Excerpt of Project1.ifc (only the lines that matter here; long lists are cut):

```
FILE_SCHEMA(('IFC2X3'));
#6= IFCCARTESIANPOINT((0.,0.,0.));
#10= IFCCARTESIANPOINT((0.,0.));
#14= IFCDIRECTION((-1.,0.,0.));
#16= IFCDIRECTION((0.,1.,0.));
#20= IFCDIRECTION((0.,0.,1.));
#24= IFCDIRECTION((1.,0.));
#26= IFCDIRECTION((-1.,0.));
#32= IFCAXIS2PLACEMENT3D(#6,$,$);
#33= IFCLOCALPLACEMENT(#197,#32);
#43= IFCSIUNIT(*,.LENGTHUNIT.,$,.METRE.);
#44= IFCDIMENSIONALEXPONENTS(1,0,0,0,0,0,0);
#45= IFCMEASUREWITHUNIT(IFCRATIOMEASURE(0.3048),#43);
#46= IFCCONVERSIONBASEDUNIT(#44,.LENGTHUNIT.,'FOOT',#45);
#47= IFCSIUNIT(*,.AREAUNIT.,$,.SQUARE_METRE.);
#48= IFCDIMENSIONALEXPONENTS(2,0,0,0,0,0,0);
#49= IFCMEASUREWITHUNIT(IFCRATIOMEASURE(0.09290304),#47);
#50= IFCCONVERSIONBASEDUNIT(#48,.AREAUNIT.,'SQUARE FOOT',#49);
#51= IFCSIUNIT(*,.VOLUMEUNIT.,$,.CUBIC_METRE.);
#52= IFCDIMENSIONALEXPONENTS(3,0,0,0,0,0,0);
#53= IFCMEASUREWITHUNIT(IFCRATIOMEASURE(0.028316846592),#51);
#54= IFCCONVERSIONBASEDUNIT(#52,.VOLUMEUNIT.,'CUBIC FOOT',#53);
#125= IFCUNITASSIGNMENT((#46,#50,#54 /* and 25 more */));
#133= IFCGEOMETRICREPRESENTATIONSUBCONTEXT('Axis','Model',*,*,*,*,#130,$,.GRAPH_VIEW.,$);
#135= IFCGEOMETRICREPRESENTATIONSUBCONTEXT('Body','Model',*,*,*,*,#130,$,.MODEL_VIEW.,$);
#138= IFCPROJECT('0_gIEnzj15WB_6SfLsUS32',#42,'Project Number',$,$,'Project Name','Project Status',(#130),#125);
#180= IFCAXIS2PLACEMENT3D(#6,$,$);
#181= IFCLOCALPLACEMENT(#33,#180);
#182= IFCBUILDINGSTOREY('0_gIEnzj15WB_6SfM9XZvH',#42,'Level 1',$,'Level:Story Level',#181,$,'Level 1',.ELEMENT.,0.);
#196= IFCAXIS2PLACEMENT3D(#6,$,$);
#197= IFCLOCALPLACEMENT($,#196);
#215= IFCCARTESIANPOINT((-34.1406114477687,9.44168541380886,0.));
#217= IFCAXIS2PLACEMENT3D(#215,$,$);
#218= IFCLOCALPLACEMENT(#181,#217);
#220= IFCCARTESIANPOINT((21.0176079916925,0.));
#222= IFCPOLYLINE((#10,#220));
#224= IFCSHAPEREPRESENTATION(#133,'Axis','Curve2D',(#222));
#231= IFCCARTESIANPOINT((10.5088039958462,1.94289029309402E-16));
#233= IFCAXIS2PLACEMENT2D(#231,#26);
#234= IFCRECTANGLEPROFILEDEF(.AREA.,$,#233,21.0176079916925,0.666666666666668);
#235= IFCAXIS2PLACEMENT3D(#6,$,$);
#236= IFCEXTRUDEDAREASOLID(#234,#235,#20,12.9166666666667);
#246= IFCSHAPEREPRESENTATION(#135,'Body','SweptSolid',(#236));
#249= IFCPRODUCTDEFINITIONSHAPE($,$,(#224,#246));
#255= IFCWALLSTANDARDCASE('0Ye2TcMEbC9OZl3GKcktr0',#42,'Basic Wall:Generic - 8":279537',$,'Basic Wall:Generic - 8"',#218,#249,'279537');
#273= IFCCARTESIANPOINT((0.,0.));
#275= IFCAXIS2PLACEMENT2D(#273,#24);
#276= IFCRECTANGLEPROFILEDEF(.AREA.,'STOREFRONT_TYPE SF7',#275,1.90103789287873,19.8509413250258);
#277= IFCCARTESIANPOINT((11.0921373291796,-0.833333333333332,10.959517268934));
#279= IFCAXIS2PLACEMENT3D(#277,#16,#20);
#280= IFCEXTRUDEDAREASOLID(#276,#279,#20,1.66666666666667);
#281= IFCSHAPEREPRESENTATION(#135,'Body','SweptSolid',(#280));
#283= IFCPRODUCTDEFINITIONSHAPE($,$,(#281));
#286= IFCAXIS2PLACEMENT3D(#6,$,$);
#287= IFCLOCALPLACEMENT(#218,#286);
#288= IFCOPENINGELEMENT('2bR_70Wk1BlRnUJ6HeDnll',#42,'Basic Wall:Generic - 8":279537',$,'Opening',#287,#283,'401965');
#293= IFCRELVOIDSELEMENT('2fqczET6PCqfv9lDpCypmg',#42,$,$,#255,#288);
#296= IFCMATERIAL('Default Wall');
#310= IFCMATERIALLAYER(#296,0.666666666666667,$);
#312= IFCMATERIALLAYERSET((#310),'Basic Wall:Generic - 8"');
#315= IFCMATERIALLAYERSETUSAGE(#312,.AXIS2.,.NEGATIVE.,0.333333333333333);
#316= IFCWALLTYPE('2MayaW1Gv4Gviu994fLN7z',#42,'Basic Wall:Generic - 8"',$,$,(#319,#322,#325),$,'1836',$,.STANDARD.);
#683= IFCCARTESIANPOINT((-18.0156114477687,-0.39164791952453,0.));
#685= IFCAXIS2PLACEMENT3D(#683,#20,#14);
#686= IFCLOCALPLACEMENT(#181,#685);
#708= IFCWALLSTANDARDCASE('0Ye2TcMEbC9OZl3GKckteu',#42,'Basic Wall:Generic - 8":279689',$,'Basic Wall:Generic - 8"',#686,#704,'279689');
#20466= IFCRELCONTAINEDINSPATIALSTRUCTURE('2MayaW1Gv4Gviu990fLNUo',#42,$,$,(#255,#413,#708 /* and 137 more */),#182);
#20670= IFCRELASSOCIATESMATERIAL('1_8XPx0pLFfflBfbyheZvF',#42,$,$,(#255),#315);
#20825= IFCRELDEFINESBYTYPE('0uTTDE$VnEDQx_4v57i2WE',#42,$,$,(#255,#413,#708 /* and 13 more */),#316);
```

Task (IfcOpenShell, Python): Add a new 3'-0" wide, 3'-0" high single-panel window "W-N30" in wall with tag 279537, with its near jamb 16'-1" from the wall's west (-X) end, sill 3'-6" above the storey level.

```python
import numpy as np
import ifcopenshell
import ifcopenshell.api.feature
import ifcopenshell.api.geometry
import ifcopenshell.api.root
import ifcopenshell.api.spatial
import ifcopenshell.api.type
import ifcopenshell.geom
import ifcopenshell.util.element
import ifcopenshell.util.placement
import ifcopenshell.util.representation
import ifcopenshell.util.shape
import ifcopenshell.util.unit

model = ifcopenshell.open("Project1.ifc")
unit_scale = ifcopenshell.util.unit.calculate_unit_scale(model)
settings = ifcopenshell.geom.settings()


def volume(element):
    """Net volume in cubic metres, openings subtracted."""
    shape = ifcopenshell.geom.create_shape(settings, element)
    return ifcopenshell.util.shape.get_volume(shape.geometry)


wall = model.by_guid("0Ye2TcMEbC9OZl3GKcktr0")
storey = ifcopenshell.util.element.get_container(wall, ifc_class="IfcBuildingStorey")
context = ifcopenshell.util.representation.get_context(model, "Model", "Body", "MODEL_VIEW")
before = volume(wall)

width, height, from_end, sill = 0.9144, 0.9144, 4.9022, 1.0668  # metres

# The wall runs along its own X axis, and the end named is its -X end.
wall_shape = ifcopenshell.geom.create_shape(settings, wall)
x, y, z = ifcopenshell.util.shape.get_vertices(wall_shape.geometry).T
start = x.min() + from_end
face, thickness = float(y.min()), float(y.max() - y.min())
wall_matrix = ifcopenshell.util.placement.get_local_placement(wall.ObjectPlacement)
level = ifcopenshell.util.placement.get_local_placement(storey.ObjectPlacement)[2, 3]


def in_wall(x, y):
    """Placement at x, y metres in the wall's axes, at sill height."""
    matrix = wall_matrix.copy()
    matrix[:, 3] = wall_matrix @ np.array([x / unit_scale, y / unit_scale, 0.0, 1.0])
    matrix[2, 3] = level + sill / unit_scale
    return matrix


# Opening: a box that overshoots both wall faces by 50 mm.
opening = ifcopenshell.api.root.create_entity(model, ifc_class="IfcOpeningElement")
box = ifcopenshell.api.geometry.add_wall_representation(
    model, context=context, length=width, height=height, thickness=thickness + 0.1
)
ifcopenshell.api.geometry.assign_representation(model, product=opening, representation=box)
ifcopenshell.api.geometry.edit_object_placement(model, product=opening, matrix=in_wall(start, face - 0.05), is_si=False)
ifcopenshell.api.feature.add_feature(model, feature=opening, element=wall)

window = ifcopenshell.api.root.create_entity(model, ifc_class="IfcWindow", name="W-N30")
window.OverallWidth, window.OverallHeight = width / unit_scale, height / unit_scale
body = ifcopenshell.api.geometry.add_window_representation(
    model,
    context=context,
    overall_width=window.OverallWidth,
    overall_height=window.OverallHeight,
    partition_type="SINGLE_PANEL",
)
ifcopenshell.api.geometry.assign_representation(model, product=window, representation=body)
ifcopenshell.api.spatial.assign_container(model, products=[window], relating_structure=storey)
fills = ifcopenshell.api.feature.add_filling(model, opening=opening, element=window)
fills.OwnerHistory = window.OwnerHistory  # required in IFC2X3

# IFC2X3 keeps the operation on the window style.
style = ifcopenshell.api.root.create_entity(model, ifc_class="IfcWindowStyle", name="W-N30")
style.OperationType, style.ConstructionType = "SINGLE_PANEL", "NOTDEFINED"
style.ParameterTakesPrecedence = style.Sizeable = False
ifcopenshell.api.type.assign_type(model, related_objects=[window], relating_type=style)

# Centre the window in the wall's thickness.
ifcopenshell.api.geometry.edit_object_placement(model, product=window, matrix=in_wall(start, face), is_si=False)
window_shape = ifcopenshell.geom.create_shape(settings, window)
depth = ifcopenshell.util.shape.get_vertices(window_shape.geometry)[:, 1]
offset = face + thickness / 2 - (depth.min() + depth.max()) / 2
ifcopenshell.api.geometry.edit_object_placement(model, product=window, matrix=in_wall(start, offset), is_si=False)

after = volume(wall)

print(f"wall volume {before:.3f} -> {after:.3f} m3")

model.write("Project1-out.ifc")
```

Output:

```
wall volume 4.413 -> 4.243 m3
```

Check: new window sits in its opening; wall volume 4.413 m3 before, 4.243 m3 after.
